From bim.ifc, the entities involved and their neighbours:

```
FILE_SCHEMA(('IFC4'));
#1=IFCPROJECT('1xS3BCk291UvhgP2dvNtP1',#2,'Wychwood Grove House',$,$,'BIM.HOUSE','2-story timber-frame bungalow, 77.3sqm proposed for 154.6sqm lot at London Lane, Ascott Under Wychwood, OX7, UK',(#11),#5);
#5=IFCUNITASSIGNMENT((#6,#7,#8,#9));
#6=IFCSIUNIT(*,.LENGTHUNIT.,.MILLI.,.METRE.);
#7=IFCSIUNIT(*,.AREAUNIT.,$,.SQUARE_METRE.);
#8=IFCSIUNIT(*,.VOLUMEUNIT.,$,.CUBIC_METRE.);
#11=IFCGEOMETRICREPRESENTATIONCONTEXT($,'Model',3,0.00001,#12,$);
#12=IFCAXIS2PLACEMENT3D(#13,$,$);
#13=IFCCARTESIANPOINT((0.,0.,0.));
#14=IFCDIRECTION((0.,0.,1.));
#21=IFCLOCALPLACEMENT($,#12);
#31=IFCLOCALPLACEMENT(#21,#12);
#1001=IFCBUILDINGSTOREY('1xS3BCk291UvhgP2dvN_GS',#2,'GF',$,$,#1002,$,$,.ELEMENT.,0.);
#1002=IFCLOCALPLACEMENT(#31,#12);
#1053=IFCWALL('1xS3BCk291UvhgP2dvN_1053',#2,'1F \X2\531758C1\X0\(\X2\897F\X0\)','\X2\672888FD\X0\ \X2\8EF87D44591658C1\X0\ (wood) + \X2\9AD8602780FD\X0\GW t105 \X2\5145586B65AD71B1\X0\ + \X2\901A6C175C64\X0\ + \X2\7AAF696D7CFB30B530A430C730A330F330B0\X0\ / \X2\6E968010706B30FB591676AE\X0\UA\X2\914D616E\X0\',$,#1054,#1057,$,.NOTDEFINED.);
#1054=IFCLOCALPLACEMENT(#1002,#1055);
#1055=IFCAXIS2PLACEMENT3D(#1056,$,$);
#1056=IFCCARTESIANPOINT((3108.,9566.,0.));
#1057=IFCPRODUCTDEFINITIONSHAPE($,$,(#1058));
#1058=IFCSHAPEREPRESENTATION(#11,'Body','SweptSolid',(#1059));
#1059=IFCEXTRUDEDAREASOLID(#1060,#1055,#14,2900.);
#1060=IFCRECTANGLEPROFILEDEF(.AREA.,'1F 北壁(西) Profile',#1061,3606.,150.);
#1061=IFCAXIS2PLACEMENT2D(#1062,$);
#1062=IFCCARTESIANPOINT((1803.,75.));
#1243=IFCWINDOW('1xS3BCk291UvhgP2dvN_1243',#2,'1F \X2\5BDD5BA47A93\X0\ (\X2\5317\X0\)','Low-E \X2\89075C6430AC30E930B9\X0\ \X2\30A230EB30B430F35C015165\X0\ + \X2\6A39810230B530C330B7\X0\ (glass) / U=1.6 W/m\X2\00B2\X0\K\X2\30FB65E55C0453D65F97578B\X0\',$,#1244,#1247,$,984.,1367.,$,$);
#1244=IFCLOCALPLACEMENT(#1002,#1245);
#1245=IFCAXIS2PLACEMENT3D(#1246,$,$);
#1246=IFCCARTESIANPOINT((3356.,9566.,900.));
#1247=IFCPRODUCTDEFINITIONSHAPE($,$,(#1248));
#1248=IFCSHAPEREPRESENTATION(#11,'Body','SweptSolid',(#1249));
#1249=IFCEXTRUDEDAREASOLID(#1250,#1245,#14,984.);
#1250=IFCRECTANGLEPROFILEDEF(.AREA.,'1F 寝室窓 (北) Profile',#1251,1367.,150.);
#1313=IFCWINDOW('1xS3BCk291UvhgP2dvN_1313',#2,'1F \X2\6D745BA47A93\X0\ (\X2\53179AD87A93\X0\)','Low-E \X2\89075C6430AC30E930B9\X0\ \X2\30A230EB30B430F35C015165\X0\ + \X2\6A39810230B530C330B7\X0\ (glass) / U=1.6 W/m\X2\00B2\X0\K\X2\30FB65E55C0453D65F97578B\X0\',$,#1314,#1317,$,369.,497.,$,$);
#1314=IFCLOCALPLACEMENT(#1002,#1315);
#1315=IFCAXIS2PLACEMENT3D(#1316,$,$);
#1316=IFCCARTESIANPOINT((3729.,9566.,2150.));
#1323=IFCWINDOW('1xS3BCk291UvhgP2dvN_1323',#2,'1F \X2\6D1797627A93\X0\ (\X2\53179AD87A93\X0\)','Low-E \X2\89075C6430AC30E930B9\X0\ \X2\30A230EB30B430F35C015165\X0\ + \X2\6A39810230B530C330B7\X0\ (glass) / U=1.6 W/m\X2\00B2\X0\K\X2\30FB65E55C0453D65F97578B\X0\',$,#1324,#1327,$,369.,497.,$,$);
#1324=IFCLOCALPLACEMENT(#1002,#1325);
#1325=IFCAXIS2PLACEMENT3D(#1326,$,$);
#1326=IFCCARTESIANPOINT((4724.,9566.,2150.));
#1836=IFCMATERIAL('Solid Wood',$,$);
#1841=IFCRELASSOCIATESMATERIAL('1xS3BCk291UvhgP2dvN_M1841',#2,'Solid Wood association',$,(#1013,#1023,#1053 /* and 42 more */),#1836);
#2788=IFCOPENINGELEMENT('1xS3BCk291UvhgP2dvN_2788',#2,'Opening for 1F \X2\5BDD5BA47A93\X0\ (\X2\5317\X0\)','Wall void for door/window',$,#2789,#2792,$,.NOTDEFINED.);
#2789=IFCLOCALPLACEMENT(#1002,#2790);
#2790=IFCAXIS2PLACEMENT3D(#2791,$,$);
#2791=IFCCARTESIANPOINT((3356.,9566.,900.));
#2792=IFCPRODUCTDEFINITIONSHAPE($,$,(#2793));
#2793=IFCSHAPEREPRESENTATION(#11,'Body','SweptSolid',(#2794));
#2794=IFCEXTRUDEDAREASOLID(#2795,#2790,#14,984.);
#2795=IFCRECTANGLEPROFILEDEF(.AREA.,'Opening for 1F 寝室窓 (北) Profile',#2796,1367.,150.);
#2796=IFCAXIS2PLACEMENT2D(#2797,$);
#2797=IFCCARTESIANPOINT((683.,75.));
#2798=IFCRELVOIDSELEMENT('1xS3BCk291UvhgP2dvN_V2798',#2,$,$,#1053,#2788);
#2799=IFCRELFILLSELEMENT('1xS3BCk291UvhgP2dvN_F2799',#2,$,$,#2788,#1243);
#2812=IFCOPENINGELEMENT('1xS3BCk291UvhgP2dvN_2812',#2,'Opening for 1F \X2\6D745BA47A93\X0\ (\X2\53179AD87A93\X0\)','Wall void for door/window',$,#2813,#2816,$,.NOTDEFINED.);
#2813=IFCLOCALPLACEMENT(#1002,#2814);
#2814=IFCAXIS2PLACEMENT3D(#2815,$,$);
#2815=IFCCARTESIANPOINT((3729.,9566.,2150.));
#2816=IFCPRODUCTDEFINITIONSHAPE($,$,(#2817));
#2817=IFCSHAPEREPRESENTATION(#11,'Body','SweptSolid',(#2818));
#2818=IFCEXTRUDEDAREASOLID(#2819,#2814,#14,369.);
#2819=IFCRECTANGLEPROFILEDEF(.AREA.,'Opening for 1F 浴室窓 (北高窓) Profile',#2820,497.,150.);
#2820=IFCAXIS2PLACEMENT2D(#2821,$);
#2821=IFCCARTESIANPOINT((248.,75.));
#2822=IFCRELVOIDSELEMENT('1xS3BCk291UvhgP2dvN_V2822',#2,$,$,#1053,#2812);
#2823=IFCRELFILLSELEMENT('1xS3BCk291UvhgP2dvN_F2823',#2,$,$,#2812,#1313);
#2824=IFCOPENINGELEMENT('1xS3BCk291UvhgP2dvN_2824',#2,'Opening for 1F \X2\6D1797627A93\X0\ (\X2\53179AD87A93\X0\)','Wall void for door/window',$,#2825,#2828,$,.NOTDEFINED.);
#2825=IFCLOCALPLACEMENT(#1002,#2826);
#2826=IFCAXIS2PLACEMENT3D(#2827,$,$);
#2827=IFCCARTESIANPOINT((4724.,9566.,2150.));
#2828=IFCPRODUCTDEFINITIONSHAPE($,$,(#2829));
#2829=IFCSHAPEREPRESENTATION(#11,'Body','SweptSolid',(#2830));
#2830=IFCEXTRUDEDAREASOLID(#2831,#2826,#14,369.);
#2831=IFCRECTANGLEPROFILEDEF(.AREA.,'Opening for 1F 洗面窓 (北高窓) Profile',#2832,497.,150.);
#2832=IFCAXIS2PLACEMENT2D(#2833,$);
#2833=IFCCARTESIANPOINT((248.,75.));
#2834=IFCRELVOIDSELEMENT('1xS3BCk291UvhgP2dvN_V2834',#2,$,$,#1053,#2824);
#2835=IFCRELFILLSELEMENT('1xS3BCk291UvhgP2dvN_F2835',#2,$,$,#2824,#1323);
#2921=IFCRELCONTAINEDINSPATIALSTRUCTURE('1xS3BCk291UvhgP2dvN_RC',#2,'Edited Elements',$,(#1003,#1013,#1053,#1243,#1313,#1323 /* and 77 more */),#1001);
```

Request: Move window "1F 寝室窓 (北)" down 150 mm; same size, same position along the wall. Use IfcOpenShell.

```python
import numpy as np
import ifcopenshell
import ifcopenshell.api.geometry
import ifcopenshell.util.placement
import ifcopenshell.util.unit

model = ifcopenshell.open("bim.ifc")
unit_scale = ifcopenshell.util.unit.calculate_unit_scale(model)

window = model.by_guid("1xS3BCk291UvhgP2dvN_1243")
opening = window.FillsVoids[0].RelatingOpeningElement
dz = -0.15 / unit_scale

shift = np.array([0.0, 0.0, dz])
# The window is not placed relative to its opening, so move both.
for product in (opening, window):
    matrix = ifcopenshell.util.placement.get_local_placement(product.ObjectPlacement)
    matrix[:3, 3] += shift
    ifcopenshell.api.geometry.edit_object_placement(model, product=product, matrix=matrix, is_si=False)

print(f"moved by {dz * unit_scale:+.3f} m")

model.write("bim-out.ifc")
```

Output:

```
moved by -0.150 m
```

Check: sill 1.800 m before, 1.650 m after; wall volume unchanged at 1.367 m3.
